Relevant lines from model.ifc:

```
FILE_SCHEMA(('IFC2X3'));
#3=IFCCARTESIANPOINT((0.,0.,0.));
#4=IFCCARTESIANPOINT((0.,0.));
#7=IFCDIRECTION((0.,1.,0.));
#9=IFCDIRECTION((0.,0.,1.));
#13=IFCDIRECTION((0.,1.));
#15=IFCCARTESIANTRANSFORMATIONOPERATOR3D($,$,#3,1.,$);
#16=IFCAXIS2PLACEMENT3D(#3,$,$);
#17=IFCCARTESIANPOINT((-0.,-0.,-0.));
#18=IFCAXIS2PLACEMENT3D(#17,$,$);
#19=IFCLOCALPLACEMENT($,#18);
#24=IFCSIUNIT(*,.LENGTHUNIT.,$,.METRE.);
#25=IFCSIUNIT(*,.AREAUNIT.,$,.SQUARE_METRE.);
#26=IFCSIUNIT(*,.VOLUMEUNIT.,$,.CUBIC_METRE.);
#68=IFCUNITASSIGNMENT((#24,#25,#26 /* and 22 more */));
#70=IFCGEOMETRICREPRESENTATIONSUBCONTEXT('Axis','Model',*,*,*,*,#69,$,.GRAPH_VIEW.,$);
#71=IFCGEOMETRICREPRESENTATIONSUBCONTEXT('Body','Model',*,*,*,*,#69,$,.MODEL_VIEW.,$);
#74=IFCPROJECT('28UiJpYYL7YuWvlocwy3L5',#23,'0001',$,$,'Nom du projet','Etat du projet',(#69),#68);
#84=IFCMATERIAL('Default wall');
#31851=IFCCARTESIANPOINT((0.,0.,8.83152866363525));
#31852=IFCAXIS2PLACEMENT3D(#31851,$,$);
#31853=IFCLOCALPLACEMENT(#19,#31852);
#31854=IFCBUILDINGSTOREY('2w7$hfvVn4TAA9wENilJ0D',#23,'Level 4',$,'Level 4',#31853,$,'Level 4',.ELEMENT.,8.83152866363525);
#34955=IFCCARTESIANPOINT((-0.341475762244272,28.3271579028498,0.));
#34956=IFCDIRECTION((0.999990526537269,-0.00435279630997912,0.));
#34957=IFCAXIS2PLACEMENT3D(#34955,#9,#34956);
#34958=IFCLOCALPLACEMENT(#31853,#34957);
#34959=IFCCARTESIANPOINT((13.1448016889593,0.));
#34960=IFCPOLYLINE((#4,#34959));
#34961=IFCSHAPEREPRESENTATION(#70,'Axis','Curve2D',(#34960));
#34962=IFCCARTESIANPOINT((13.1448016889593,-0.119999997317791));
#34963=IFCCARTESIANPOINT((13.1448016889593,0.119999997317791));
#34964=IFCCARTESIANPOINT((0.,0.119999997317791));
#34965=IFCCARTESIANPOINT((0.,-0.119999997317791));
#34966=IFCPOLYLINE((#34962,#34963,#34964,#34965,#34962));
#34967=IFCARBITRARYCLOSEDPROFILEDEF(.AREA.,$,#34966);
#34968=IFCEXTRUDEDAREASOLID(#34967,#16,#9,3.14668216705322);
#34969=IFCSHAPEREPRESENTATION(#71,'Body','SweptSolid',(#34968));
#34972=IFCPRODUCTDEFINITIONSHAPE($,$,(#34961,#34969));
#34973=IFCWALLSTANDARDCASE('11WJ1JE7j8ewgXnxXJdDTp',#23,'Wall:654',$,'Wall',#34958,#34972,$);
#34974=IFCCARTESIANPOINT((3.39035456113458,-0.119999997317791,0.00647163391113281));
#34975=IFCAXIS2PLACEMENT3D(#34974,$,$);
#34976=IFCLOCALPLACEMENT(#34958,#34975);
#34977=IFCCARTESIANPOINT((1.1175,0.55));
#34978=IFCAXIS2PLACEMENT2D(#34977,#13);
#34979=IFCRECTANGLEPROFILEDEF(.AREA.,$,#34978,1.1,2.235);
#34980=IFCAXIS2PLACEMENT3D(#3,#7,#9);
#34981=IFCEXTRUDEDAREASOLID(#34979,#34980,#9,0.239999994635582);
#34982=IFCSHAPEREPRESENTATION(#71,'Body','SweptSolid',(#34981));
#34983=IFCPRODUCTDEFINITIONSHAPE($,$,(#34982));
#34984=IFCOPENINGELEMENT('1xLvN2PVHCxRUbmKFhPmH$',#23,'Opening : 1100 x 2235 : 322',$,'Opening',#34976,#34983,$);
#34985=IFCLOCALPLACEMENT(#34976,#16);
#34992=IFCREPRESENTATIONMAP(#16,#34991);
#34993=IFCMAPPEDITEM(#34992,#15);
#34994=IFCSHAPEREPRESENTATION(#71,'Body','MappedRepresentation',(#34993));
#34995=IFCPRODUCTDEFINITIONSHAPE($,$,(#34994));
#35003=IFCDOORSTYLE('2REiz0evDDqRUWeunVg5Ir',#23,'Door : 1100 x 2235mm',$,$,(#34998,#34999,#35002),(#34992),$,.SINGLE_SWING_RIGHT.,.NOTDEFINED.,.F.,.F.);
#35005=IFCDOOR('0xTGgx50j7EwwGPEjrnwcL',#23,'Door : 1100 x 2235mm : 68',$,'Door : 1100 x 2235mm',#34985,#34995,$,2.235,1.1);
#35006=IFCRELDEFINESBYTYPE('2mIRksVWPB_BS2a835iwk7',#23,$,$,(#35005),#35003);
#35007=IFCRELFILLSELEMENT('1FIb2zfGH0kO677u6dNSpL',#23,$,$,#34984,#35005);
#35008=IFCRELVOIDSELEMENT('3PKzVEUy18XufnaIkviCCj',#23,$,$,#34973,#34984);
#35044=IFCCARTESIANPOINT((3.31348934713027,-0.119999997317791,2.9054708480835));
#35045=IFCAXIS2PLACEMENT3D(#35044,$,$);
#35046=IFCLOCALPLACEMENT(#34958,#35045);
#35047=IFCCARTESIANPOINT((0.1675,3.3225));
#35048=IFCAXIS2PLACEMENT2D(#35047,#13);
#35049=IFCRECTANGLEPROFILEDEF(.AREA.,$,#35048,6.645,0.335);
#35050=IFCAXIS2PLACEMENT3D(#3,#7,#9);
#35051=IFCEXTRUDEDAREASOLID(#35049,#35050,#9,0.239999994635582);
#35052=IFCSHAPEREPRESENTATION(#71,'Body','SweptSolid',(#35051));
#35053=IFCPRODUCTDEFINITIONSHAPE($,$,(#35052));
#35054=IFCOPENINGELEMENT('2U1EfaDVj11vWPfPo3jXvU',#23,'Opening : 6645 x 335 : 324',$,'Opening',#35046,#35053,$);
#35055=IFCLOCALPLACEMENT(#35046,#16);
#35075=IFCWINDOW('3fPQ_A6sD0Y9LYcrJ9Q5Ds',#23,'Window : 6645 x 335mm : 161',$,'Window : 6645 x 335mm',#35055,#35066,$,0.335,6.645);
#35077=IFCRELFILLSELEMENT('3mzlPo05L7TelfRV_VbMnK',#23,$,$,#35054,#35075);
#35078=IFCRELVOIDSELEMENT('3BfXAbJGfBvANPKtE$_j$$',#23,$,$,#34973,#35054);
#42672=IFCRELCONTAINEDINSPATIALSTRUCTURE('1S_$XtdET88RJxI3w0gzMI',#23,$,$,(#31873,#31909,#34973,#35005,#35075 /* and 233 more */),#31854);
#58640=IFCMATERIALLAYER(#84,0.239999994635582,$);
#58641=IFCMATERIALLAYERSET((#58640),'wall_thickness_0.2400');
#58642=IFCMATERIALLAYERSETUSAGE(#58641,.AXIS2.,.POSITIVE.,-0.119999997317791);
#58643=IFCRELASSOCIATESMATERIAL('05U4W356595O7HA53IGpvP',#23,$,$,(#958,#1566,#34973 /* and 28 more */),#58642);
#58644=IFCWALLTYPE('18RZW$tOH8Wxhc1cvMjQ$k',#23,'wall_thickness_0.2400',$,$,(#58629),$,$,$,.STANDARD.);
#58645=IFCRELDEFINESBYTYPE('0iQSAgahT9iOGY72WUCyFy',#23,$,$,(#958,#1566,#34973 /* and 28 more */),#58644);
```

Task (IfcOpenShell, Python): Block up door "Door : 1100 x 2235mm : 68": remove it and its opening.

```python
import ifcopenshell
import ifcopenshell.api.feature
import ifcopenshell.api.root
import ifcopenshell.geom
import ifcopenshell.util.shape

model = ifcopenshell.open("model.ifc")
settings = ifcopenshell.geom.settings()


def volume(element):
    """Net volume in cubic metres, openings subtracted."""
    shape = ifcopenshell.geom.create_shape(settings, element)
    return ifcopenshell.util.shape.get_volume(shape.geometry)


door = model.by_id(35005)
opening = door.FillsVoids[0].RelatingOpeningElement
wall = opening.VoidsElements[0].RelatingBuildingElement
before = volume(wall)

ifcopenshell.api.root.remove_product(model, product=door)
ifcopenshell.api.feature.remove_feature(model, feature=opening)

after = volume(wall)

print(f"wall volume {before:.3f} -> {after:.3f} m3")

model.write("model-out.ifc")
```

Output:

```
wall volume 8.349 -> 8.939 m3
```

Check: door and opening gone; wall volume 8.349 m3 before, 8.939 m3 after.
